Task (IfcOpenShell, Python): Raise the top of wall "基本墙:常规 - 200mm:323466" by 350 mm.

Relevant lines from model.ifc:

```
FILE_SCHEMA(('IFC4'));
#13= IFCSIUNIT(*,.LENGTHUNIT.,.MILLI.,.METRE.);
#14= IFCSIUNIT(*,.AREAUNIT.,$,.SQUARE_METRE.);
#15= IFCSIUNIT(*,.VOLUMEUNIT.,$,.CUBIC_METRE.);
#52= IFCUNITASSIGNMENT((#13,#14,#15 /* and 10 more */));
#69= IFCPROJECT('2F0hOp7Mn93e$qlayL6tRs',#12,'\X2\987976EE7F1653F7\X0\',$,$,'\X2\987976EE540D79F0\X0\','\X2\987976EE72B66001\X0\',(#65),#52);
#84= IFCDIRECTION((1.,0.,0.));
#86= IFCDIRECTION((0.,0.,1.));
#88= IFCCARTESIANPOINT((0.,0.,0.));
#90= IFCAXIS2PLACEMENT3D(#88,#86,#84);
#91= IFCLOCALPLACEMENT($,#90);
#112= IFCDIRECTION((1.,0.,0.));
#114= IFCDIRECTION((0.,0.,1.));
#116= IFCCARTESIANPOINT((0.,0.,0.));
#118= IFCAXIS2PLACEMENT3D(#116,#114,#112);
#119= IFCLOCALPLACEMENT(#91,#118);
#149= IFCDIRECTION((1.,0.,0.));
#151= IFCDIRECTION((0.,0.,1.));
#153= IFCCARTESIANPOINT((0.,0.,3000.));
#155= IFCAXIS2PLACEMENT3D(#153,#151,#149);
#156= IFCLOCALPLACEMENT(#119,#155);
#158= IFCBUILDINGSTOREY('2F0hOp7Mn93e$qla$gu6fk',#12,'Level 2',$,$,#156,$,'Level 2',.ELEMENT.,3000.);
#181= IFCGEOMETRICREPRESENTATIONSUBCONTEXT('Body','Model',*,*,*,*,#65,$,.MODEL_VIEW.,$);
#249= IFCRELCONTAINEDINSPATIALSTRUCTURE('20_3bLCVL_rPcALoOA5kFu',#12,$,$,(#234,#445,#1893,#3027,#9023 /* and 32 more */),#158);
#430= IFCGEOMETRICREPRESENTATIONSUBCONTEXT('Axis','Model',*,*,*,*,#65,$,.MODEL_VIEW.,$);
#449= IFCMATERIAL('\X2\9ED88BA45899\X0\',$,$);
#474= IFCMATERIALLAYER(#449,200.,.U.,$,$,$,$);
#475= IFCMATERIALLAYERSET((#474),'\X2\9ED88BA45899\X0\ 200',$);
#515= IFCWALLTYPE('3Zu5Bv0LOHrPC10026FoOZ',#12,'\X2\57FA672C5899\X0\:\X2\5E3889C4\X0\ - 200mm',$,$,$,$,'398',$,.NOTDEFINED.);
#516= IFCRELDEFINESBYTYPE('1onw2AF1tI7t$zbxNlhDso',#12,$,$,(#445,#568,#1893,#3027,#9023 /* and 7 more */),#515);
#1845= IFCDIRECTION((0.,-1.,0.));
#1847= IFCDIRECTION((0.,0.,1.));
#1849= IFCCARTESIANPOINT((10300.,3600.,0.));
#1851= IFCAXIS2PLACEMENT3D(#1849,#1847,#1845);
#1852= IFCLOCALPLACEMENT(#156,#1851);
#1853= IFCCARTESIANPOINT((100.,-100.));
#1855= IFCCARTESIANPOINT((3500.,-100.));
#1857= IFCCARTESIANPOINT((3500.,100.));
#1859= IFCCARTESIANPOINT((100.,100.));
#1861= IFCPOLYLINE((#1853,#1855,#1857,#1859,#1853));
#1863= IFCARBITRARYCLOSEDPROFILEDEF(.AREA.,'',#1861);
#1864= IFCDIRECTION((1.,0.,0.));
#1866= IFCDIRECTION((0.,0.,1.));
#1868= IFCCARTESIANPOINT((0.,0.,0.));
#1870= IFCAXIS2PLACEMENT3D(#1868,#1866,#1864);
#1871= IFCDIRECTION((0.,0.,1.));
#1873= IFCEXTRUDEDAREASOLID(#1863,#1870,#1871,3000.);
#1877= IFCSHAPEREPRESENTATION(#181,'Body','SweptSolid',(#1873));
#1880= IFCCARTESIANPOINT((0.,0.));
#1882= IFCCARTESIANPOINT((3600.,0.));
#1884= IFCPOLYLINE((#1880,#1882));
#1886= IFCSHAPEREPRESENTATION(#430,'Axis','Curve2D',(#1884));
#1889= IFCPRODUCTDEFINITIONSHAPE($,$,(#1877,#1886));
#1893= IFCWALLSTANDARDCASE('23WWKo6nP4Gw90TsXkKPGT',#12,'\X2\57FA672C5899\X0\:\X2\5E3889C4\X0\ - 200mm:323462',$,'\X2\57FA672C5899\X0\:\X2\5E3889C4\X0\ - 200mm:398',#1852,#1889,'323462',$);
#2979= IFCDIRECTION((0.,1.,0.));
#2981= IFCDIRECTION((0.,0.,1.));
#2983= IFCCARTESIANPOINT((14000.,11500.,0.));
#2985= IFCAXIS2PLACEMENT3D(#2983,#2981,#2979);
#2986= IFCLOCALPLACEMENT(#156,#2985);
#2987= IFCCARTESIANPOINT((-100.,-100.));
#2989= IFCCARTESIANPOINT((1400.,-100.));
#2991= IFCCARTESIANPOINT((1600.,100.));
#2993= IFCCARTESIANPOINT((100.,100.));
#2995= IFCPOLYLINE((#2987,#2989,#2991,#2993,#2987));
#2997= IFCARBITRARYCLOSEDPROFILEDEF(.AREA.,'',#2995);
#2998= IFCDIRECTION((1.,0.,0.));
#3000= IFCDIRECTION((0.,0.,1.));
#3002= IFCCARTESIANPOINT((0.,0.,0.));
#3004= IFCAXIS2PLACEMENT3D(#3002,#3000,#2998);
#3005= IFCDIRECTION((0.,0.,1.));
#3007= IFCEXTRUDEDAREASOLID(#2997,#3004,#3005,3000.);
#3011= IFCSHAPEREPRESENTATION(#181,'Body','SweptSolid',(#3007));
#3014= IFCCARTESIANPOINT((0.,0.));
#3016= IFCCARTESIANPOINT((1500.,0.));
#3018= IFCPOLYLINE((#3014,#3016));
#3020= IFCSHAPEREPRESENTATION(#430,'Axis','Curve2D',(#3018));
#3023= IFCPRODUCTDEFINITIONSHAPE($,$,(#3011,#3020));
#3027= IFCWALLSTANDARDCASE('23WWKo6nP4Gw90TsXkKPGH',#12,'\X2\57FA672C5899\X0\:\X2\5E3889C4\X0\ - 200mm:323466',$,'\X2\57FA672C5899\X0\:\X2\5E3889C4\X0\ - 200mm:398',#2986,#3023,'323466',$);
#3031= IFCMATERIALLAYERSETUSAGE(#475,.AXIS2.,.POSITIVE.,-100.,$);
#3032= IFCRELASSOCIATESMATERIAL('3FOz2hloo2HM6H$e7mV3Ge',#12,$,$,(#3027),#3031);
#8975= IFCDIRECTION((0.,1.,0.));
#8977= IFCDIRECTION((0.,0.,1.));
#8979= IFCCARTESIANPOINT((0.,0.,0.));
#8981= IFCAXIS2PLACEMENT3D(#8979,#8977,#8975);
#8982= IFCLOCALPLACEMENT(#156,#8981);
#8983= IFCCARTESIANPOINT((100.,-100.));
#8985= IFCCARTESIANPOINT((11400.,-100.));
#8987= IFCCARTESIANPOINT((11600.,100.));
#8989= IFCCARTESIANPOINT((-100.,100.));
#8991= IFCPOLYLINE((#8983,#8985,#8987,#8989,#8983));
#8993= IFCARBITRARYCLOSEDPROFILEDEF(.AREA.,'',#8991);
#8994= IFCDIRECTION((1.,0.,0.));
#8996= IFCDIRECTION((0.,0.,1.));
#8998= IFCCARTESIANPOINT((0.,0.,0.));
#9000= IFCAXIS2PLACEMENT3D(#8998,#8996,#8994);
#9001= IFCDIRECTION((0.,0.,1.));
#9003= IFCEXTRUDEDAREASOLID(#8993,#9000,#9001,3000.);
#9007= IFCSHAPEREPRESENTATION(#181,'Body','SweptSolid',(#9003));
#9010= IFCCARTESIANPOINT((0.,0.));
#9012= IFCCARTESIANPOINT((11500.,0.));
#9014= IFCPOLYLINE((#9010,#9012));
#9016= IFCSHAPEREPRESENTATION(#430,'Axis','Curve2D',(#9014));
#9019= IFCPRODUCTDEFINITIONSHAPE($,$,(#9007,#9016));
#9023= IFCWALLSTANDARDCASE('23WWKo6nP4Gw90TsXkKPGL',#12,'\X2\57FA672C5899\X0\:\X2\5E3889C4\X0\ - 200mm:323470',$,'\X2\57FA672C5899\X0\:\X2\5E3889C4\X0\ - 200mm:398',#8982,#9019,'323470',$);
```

```python
import ifcopenshell
import ifcopenshell.geom
import ifcopenshell.util.representation
import ifcopenshell.util.shape
import ifcopenshell.util.unit

model = ifcopenshell.open("model.ifc")
unit_scale = ifcopenshell.util.unit.calculate_unit_scale(model)
settings = ifcopenshell.geom.settings()


def volume(element):
    """Net volume in cubic metres, openings subtracted."""
    shape = ifcopenshell.geom.create_shape(settings, element)
    return ifcopenshell.util.shape.get_volume(shape.geometry)


wall = model.by_guid("23WWKo6nP4Gw90TsXkKPGH")
before = volume(wall)

body = ifcopenshell.util.representation.get_representation(wall, "Model", "Body")
solid = body.Items[0]
old_height = solid.Depth
solid.Depth += 0.35 / unit_scale
after = volume(wall)

print(f"height {old_height:g} -> {solid.Depth:g}, volume {before:.3f} -> {after:.3f} m3")

model.write("model-out.ifc")
```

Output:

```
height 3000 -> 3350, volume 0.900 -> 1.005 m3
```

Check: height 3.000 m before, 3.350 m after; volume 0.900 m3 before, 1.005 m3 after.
